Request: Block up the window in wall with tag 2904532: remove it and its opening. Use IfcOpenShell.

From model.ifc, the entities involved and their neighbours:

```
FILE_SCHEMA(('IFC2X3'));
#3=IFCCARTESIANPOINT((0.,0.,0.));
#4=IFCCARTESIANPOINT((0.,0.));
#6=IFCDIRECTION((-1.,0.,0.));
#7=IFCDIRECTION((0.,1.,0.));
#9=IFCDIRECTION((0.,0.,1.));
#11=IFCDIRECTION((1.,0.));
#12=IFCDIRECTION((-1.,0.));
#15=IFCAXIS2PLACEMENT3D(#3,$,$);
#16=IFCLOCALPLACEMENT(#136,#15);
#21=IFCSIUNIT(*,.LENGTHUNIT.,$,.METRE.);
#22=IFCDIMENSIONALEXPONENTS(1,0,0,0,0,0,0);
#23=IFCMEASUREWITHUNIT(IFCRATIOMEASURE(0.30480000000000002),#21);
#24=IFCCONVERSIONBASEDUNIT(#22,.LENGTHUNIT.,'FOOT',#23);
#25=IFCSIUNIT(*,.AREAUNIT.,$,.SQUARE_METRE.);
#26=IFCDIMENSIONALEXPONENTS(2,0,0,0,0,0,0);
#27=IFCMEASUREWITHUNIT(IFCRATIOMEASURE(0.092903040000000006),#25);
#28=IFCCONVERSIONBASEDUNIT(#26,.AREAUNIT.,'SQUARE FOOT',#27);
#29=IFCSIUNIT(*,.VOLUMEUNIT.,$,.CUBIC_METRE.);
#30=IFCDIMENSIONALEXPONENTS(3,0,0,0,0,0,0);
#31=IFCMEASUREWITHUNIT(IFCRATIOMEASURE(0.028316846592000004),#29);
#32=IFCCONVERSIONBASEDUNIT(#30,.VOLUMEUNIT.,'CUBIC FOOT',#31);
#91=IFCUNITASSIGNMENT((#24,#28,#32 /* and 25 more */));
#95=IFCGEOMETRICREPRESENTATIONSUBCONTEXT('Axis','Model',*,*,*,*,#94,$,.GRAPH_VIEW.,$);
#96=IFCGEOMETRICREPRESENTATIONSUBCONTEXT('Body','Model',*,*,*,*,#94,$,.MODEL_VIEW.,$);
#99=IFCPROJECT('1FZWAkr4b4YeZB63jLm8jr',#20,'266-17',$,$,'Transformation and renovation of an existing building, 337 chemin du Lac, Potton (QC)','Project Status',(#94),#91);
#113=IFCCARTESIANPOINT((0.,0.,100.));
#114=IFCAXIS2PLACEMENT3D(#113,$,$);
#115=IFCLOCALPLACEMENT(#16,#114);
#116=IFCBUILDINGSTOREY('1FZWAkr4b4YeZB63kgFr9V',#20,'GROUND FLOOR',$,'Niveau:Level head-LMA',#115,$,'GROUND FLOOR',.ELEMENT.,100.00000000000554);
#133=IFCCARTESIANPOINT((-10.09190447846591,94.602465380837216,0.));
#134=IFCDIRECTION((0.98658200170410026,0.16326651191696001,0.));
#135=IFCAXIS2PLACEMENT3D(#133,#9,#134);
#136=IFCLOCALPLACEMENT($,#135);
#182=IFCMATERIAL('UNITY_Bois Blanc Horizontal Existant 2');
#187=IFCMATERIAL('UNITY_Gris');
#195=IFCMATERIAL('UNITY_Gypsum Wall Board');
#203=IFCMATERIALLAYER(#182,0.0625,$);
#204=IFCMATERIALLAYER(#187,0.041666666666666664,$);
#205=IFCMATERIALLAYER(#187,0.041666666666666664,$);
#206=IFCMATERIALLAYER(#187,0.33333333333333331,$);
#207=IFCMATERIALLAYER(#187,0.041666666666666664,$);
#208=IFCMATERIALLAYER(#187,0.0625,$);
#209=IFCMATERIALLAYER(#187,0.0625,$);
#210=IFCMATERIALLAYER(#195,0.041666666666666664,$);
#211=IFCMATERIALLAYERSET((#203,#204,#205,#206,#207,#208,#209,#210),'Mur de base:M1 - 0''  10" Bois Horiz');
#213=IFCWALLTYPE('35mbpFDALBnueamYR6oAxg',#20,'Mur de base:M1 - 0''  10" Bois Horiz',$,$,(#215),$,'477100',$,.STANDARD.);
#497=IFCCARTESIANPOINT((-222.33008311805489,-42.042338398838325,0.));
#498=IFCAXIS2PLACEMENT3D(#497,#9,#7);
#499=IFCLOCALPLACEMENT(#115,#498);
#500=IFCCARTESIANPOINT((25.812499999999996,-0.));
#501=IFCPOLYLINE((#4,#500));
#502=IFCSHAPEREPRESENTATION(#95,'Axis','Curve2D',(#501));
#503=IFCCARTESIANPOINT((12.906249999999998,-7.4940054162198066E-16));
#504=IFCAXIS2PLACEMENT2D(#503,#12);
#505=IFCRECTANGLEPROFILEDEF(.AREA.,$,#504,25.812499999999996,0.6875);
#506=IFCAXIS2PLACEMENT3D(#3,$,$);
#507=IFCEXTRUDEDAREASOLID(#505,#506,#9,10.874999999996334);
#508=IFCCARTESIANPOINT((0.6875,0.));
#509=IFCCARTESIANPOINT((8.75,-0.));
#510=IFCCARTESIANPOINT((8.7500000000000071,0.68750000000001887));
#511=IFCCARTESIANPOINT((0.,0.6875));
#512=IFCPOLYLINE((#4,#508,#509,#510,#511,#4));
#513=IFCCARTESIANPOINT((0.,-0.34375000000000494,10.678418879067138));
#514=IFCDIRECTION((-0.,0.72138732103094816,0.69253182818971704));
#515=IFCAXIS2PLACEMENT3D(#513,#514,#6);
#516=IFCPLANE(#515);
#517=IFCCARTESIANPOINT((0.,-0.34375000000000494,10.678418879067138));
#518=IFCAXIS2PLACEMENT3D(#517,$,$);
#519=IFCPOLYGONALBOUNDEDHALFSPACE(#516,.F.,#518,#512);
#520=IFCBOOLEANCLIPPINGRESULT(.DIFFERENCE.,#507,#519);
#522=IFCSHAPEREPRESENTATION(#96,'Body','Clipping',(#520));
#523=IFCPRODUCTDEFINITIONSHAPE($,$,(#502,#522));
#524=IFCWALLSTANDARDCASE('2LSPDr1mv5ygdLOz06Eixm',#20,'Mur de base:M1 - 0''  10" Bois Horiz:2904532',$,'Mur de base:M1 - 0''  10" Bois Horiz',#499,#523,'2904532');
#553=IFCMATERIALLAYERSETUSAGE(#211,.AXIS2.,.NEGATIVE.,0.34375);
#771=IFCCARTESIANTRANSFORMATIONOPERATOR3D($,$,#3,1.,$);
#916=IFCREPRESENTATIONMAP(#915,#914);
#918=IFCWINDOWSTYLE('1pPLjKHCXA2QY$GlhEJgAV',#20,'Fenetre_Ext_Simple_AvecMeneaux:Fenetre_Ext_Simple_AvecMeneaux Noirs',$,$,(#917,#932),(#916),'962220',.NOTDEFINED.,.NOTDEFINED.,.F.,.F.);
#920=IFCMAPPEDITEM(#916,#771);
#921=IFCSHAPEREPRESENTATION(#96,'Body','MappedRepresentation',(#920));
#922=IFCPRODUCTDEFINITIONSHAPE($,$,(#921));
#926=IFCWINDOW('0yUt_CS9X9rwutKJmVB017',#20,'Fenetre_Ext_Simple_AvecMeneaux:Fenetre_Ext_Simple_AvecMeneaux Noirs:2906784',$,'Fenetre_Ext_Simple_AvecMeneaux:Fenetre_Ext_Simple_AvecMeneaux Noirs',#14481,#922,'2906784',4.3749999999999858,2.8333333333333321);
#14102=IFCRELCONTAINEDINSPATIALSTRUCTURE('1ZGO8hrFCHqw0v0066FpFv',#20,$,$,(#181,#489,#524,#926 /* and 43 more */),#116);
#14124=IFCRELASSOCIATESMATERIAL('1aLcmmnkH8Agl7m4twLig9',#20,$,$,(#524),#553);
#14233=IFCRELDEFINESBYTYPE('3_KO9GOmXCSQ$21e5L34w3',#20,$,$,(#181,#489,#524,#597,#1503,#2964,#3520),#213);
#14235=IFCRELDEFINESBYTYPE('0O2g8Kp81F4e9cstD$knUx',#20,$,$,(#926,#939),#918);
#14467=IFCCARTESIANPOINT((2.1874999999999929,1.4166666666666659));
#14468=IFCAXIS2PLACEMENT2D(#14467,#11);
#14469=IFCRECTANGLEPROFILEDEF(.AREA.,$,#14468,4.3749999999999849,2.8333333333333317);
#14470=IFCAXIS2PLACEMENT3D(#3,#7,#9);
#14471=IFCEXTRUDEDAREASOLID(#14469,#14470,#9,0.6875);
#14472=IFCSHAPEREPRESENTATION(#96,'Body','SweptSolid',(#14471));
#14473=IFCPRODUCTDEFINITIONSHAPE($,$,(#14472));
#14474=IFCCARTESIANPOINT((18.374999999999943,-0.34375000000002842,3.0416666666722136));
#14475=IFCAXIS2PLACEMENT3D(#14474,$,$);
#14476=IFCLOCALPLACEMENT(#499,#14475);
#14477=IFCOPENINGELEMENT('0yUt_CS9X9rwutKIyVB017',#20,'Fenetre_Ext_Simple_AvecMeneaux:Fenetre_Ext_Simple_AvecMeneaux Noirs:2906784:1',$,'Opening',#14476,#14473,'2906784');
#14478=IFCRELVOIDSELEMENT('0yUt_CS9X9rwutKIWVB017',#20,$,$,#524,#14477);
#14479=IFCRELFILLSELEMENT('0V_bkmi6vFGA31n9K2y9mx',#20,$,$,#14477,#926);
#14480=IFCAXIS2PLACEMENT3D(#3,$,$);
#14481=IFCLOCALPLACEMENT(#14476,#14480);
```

```python
import ifcopenshell
import ifcopenshell.api.feature
import ifcopenshell.api.root
import ifcopenshell.geom
import ifcopenshell.util.shape

model = ifcopenshell.open("model.ifc")
settings = ifcopenshell.geom.settings()


def volume(element):
    """Net volume in cubic metres, openings subtracted."""
    shape = ifcopenshell.geom.create_shape(settings, element)
    return ifcopenshell.util.shape.get_volume(shape.geometry)


window = model.by_guid("0yUt_CS9X9rwutKJmVB017")
opening = window.FillsVoids[0].RelatingOpeningElement
wall = opening.VoidsElements[0].RelatingBuildingElement
before = volume(wall)

ifcopenshell.api.root.remove_product(model, product=window)
ifcopenshell.api.feature.remove_feature(model, feature=opening)

after = volume(wall)

print(f"wall volume {before:.3f} -> {after:.3f} m3")

model.write("model_updated.ifc")
```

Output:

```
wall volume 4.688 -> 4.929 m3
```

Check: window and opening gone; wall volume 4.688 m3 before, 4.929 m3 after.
